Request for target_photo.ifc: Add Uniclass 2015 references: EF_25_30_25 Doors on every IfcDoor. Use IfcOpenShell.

First a look at what the model holds.

```python
import ifcopenshell

model = ifcopenshell.open("target_photo.ifc")
print(model.schema)
print("classifications:", [c.Name for c in model.by_type("IfcClassification")])
for ifc_class in ("IfcDoor", "IfcRoof", "IfcStair", "IfcWall", "IfcWindow"):
    print(ifc_class, len(model.by_type(ifc_class)))
```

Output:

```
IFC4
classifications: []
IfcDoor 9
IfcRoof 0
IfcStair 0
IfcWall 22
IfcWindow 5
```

```python
import ifcopenshell
import ifcopenshell.api.classification

model = ifcopenshell.open("target_photo.ifc")

system = ifcopenshell.api.classification.add_classification(model, classification="Uniclass 2015")

codes = {
    "IfcDoor": ("EF_25_30_25", "Doors"),
}
for ifc_class, (code, name) in codes.items():
    products = model.by_type(ifc_class)
    ifcopenshell.api.classification.add_reference(
        model, products=products, classification=system, identification=code, name=name
    )
    print(code, len(products))

model.write("target_photo_updated.ifc")
```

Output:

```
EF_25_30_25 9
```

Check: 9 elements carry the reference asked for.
